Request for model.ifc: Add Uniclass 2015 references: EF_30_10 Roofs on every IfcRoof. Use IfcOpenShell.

First a look at what the model holds.

```python
import ifcopenshell

model = ifcopenshell.open("model.ifc")
print(model.schema)
print("classifications:", [c.Name for c in model.by_type("IfcClassification")])
for ifc_class in ("IfcDoor", "IfcRoof", "IfcStair", "IfcWall", "IfcWindow"):
    print(ifc_class, len(model.by_type(ifc_class)))
```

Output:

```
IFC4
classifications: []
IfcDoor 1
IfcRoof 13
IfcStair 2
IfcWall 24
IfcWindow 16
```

```python
import ifcopenshell
import ifcopenshell.api.classification

model = ifcopenshell.open("model.ifc")

system = ifcopenshell.api.classification.add_classification(model, classification="Uniclass 2015")

codes = {
    "IfcRoof": ("EF_30_10", "Roofs"),
}
for ifc_class, (code, name) in codes.items():
    products = model.by_type(ifc_class)
    ifcopenshell.api.classification.add_reference(
        model, products=products, classification=system, identification=code, name=name
    )
    print(code, len(products))

model.write("model_v2.ifc")
```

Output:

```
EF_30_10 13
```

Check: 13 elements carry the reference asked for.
